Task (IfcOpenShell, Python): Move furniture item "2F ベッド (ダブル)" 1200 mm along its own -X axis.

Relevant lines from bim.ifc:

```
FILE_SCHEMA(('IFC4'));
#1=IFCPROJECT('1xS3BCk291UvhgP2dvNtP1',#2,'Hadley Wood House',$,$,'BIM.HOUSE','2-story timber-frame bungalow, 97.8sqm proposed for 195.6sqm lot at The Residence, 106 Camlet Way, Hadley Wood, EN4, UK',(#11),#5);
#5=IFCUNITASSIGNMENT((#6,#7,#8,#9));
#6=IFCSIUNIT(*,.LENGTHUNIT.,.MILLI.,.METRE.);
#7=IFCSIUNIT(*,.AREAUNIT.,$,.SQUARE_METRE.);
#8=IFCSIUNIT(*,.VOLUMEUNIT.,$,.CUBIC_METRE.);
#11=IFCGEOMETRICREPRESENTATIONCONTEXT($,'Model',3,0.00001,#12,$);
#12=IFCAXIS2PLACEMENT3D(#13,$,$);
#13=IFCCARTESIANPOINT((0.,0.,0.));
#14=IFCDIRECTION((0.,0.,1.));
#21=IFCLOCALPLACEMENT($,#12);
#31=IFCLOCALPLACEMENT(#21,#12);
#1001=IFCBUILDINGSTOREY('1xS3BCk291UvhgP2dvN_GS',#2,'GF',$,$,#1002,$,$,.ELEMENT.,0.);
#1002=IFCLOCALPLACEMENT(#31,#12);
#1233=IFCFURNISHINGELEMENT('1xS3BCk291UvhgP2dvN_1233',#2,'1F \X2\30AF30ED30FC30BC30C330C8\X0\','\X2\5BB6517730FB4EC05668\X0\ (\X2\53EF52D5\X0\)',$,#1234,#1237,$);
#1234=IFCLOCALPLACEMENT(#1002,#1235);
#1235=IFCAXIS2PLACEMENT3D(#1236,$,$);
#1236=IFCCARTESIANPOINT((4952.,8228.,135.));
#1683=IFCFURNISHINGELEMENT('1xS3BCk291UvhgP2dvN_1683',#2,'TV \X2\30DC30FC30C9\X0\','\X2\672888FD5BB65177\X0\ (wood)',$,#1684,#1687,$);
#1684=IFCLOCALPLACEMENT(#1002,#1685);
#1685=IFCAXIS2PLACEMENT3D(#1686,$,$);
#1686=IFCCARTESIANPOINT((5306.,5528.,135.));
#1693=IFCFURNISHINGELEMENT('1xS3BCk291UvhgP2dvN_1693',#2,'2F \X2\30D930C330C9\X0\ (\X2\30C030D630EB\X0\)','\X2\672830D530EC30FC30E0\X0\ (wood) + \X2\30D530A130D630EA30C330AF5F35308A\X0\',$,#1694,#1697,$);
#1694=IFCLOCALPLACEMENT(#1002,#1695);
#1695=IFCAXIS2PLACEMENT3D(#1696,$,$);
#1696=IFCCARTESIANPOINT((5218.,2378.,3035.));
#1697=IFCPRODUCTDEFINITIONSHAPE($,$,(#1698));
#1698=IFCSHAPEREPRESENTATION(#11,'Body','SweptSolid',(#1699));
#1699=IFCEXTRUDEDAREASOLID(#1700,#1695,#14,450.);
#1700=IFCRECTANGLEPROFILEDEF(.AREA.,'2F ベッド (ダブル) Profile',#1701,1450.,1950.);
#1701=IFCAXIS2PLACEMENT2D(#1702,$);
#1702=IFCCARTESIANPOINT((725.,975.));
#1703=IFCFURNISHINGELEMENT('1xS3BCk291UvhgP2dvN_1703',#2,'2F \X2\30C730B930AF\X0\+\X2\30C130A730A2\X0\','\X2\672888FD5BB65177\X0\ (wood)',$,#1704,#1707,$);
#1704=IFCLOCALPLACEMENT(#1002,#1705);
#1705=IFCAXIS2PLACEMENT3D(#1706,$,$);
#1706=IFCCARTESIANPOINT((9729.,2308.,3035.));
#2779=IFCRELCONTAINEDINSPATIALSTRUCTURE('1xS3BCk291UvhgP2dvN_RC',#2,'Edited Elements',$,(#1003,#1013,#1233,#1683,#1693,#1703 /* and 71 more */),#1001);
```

```python
import ifcopenshell
import ifcopenshell.api.geometry
import ifcopenshell.util.placement
import ifcopenshell.util.unit

model = ifcopenshell.open("bim.ifc")
unit_scale = ifcopenshell.util.unit.calculate_unit_scale(model)

item = model.by_guid("1xS3BCk291UvhgP2dvN_1693")
matrix = ifcopenshell.util.placement.get_local_placement(item.ObjectPlacement)
matrix[:3, 3] -= matrix[:3, 0] * 1.2 / unit_scale
ifcopenshell.api.geometry.edit_object_placement(model, product=item, matrix=matrix, is_si=False)

print(ifcopenshell.util.placement.get_local_placement(item.ObjectPlacement).round(3) + 0.0)

model.write("bim_v2.ifc")
```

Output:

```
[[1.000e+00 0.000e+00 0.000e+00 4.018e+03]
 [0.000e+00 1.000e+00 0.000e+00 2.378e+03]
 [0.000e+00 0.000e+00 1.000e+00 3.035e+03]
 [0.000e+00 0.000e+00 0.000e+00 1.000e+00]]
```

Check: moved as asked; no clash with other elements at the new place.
